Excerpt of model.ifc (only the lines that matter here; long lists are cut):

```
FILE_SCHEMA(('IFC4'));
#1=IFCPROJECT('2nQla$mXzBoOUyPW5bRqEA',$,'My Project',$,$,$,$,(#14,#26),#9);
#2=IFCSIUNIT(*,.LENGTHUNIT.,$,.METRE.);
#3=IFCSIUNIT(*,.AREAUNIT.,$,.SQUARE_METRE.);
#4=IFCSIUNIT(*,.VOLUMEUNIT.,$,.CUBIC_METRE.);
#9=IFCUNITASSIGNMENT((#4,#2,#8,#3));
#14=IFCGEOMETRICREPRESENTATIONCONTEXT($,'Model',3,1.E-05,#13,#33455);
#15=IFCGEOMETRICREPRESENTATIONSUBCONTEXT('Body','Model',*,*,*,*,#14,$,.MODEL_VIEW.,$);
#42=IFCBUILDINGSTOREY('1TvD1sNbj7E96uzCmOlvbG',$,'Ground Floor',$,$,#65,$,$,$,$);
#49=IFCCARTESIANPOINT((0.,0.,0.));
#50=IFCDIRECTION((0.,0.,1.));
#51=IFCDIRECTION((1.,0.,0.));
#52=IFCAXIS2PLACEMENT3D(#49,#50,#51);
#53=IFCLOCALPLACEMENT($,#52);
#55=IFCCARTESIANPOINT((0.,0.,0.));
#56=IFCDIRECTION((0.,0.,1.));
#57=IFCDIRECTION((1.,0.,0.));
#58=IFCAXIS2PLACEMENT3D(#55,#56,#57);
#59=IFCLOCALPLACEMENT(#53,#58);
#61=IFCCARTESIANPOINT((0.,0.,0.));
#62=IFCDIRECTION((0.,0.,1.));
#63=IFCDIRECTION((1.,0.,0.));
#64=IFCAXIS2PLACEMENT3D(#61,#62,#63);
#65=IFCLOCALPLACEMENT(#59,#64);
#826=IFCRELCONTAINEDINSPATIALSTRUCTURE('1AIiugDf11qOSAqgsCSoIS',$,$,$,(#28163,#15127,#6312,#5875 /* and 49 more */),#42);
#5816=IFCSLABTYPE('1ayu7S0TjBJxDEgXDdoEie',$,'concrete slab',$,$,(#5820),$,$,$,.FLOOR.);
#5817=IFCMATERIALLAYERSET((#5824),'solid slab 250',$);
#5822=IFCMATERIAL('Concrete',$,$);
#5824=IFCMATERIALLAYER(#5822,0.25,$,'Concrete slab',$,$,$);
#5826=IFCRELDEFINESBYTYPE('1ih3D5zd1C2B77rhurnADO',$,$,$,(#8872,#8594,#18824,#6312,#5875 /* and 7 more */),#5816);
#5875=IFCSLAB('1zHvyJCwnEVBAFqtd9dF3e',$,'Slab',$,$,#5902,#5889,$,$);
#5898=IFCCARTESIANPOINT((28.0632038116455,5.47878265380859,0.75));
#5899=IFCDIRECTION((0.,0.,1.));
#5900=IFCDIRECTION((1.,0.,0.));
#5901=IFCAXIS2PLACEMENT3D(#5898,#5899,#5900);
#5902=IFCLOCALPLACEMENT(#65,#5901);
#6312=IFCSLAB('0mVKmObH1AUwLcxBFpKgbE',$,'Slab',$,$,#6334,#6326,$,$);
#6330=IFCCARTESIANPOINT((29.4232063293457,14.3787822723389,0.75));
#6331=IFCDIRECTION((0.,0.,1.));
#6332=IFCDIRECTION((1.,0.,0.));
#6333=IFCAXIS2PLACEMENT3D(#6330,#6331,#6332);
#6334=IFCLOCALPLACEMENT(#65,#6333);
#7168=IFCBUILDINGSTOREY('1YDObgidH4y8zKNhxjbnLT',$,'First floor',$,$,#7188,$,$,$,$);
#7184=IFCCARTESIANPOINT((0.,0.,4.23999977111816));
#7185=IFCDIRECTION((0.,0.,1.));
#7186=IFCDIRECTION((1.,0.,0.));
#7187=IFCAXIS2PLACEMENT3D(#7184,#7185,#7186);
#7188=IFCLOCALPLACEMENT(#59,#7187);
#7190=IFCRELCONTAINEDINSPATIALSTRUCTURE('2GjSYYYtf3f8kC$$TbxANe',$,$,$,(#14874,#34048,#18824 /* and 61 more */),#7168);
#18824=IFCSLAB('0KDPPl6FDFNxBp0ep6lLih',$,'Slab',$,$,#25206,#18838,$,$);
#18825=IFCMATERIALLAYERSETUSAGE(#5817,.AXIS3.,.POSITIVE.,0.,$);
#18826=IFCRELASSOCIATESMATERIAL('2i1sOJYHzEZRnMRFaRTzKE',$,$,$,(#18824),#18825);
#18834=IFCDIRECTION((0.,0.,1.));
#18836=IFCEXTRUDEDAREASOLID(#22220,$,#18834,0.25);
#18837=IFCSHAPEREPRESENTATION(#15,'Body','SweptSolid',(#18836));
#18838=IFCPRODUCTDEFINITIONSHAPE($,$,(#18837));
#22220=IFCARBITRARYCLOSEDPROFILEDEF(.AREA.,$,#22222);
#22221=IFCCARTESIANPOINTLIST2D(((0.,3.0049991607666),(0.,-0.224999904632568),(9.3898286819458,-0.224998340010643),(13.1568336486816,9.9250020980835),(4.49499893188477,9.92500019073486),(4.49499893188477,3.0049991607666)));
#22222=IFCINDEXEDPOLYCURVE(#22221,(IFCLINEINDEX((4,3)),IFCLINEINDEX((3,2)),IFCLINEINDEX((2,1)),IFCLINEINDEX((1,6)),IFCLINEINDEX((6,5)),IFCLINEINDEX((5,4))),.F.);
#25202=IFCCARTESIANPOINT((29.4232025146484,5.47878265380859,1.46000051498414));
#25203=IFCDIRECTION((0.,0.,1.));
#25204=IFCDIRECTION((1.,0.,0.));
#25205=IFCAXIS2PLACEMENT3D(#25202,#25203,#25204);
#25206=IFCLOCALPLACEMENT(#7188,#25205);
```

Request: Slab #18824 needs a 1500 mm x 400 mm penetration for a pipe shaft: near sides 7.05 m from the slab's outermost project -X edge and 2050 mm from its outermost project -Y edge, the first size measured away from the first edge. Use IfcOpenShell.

```python
import numpy as np
import ifcopenshell
import ifcopenshell.api.feature
import ifcopenshell.api.geometry
import ifcopenshell.api.root
import ifcopenshell.geom
import ifcopenshell.util.placement
import ifcopenshell.util.representation
import ifcopenshell.util.shape
import ifcopenshell.util.unit

model = ifcopenshell.open("model.ifc")
unit_scale = ifcopenshell.util.unit.calculate_unit_scale(model)
settings = ifcopenshell.geom.settings()


def volume(element):
    """Net volume in cubic metres, openings subtracted."""
    shape = ifcopenshell.geom.create_shape(settings, element)
    return ifcopenshell.util.shape.get_volume(shape.geometry)


slab = model.by_id(18824)
before = volume(slab)

# Extent in the slab's own axes, in metres. The edges named are its -X and -Y sides.
slab_shape = ifcopenshell.geom.create_shape(settings, slab)
vertices = ifcopenshell.util.shape.get_vertices(slab_shape.geometry)
x_min, y_min, bottom = vertices.min(axis=0)
top = vertices[:, 2].max()

opening = ifcopenshell.api.root.create_entity(model, ifc_class="IfcOpeningElement", name="Pipe shaft opening", predefined_type="OPENING")
context = ifcopenshell.util.representation.get_context(model, "Model", "Body", "MODEL_VIEW")
width, depth = 1.5, 0.4
outline = [(0.0, 0.0), (width, 0.0), (width, depth), (0.0, depth), (0.0, 0.0)]
# Overshoot both faces by 50 mm so the cut is clean.
shape = ifcopenshell.api.geometry.add_slab_representation(
    model, context=context, depth=top - bottom + 0.1, polyline=outline
)
ifcopenshell.api.geometry.assign_representation(model, product=opening, representation=shape)

matrix = ifcopenshell.util.placement.get_local_placement(slab.ObjectPlacement)
matrix[:, 3] = matrix @ np.append(np.array([x_min + 7.05, y_min + 2.05, bottom - 0.05]) / unit_scale, 1.0)
ifcopenshell.api.geometry.edit_object_placement(model, product=opening, matrix=matrix, is_si=False)
ifcopenshell.api.feature.add_feature(model, feature=opening, element=slab)

after = volume(slab)

print(f"slab volume {before:.3f} -> {after:.3f} m3")

model.write("model_v2.ifc")
```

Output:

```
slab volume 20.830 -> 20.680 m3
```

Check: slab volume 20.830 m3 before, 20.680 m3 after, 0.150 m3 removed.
